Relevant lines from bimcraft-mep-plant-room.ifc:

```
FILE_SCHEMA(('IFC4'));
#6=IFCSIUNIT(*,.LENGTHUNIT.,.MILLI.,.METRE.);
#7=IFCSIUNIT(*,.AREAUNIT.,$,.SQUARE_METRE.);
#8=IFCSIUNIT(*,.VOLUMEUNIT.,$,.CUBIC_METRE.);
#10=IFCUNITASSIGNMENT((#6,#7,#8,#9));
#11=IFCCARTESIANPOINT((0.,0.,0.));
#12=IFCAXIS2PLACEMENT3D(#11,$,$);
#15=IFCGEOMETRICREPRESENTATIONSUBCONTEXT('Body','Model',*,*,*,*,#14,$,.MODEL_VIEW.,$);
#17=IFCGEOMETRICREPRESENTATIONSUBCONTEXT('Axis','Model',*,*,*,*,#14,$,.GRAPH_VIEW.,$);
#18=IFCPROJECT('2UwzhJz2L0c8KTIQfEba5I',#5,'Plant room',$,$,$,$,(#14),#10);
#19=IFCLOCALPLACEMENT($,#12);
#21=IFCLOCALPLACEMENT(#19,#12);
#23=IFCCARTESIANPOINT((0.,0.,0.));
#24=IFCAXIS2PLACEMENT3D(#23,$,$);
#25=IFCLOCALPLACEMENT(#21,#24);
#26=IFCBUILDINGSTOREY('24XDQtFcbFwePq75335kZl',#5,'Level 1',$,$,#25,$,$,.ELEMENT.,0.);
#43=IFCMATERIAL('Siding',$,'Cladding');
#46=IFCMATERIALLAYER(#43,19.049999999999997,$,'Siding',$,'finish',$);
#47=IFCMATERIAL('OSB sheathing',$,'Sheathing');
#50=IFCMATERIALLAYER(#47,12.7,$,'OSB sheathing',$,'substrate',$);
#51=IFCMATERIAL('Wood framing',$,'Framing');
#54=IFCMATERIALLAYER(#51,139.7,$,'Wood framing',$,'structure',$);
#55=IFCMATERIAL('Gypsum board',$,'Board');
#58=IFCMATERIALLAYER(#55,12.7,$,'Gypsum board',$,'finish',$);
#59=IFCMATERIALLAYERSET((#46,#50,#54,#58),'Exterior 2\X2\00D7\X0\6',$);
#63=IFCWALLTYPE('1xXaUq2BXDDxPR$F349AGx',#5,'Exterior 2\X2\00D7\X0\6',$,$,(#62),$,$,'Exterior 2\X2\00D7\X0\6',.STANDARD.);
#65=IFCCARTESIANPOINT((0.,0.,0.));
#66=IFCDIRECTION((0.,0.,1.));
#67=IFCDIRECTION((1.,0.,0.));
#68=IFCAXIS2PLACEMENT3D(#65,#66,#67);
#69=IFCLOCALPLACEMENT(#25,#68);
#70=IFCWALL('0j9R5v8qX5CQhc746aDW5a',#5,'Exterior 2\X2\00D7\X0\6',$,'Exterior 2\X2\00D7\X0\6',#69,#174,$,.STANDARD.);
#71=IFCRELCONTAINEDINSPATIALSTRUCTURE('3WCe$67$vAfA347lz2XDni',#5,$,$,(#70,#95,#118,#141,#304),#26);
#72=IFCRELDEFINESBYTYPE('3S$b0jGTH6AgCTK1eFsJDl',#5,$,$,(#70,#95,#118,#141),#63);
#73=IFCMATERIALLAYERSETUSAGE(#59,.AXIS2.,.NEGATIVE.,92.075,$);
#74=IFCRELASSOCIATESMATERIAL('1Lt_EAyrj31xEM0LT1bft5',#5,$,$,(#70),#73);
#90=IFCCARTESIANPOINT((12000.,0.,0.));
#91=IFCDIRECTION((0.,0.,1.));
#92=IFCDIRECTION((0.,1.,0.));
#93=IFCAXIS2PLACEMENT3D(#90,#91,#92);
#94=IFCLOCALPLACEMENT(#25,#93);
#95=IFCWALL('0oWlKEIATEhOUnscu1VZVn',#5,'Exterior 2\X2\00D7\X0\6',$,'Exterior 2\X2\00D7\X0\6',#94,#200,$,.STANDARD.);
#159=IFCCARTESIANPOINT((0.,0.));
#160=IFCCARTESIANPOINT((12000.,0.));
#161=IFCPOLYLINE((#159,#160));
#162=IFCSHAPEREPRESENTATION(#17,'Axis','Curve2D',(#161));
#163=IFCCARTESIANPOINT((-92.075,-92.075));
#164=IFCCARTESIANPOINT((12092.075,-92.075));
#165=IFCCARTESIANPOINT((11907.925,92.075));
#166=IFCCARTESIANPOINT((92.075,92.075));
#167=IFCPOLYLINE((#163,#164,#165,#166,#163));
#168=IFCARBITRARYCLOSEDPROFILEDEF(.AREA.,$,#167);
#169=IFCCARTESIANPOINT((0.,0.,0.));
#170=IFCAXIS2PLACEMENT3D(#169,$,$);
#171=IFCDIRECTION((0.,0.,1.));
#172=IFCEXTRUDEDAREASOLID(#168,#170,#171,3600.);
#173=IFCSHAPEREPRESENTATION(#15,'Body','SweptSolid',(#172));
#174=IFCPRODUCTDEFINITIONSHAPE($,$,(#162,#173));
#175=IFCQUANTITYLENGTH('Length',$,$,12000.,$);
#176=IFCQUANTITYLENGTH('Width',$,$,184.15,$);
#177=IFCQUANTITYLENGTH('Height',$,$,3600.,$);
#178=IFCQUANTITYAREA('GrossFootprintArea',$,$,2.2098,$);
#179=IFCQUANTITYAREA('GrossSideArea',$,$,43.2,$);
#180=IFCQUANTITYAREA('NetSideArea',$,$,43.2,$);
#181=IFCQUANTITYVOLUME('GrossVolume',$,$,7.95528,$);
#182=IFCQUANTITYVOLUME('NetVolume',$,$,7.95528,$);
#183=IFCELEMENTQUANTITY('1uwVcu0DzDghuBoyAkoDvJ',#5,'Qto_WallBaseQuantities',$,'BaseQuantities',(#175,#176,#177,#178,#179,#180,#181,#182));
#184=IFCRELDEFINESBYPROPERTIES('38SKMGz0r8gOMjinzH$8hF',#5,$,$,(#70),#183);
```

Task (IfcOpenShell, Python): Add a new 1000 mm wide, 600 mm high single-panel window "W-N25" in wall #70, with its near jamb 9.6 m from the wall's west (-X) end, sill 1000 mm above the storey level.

```python
import numpy as np
import ifcopenshell
import ifcopenshell.api.feature
import ifcopenshell.api.geometry
import ifcopenshell.api.pset
import ifcopenshell.api.root
import ifcopenshell.api.spatial
import ifcopenshell.geom
import ifcopenshell.util.element
import ifcopenshell.util.placement
import ifcopenshell.util.representation
import ifcopenshell.util.shape
import ifcopenshell.util.unit

model = ifcopenshell.open("bimcraft-mep-plant-room.ifc")
unit_scale = ifcopenshell.util.unit.calculate_unit_scale(model)
area_scale = ifcopenshell.util.unit.calculate_unit_scale(model, "AREAUNIT")
volume_scale = ifcopenshell.util.unit.calculate_unit_scale(model, "VOLUMEUNIT")
settings = ifcopenshell.geom.settings()


def volume(element):
    """Net volume in cubic metres, openings subtracted."""
    shape = ifcopenshell.geom.create_shape(settings, element)
    return ifcopenshell.util.shape.get_volume(shape.geometry)


wall = model.by_guid("0j9R5v8qX5CQhc746aDW5a")
storey = ifcopenshell.util.element.get_container(wall, ifc_class="IfcBuildingStorey")
context = ifcopenshell.util.representation.get_context(model, "Model", "Body", "MODEL_VIEW")
before = volume(wall)

width, height, from_end, sill = 1, 0.6, 9.6, 1  # metres

# The wall runs along its own X axis, and the end named is its -X end.
wall_shape = ifcopenshell.geom.create_shape(settings, wall)
x, y, z = ifcopenshell.util.shape.get_vertices(wall_shape.geometry).T
start = x.min() + from_end
face, thickness = float(y.min()), float(y.max() - y.min())
wall_matrix = ifcopenshell.util.placement.get_local_placement(wall.ObjectPlacement)
level = ifcopenshell.util.placement.get_local_placement(storey.ObjectPlacement)[2, 3]


def in_wall(x, y):
    """Placement at x, y metres in the wall's axes, at sill height."""
    matrix = wall_matrix.copy()
    matrix[:, 3] = wall_matrix @ np.array([x / unit_scale, y / unit_scale, 0.0, 1.0])
    matrix[2, 3] = level + sill / unit_scale
    return matrix


# Opening: a box that overshoots both wall faces by 50 mm.
opening = ifcopenshell.api.root.create_entity(model, ifc_class="IfcOpeningElement", predefined_type="OPENING")
box = ifcopenshell.api.geometry.add_wall_representation(
    model, context=context, length=width, height=height, thickness=thickness + 0.1
)
ifcopenshell.api.geometry.assign_representation(model, product=opening, representation=box)
ifcopenshell.api.geometry.edit_object_placement(model, product=opening, matrix=in_wall(start, face - 0.05), is_si=False)
ifcopenshell.api.feature.add_feature(model, feature=opening, element=wall)

window = ifcopenshell.api.root.create_entity(model, ifc_class="IfcWindow", name="W-N25", predefined_type="WINDOW")
window.OverallWidth, window.OverallHeight = width / unit_scale, height / unit_scale
window.PartitioningType = "SINGLE_PANEL"
body = ifcopenshell.api.geometry.add_window_representation(
    model,
    context=context,
    overall_width=window.OverallWidth,
    overall_height=window.OverallHeight,
    partition_type="SINGLE_PANEL",
)
ifcopenshell.api.geometry.assign_representation(model, product=window, representation=body)
ifcopenshell.api.spatial.assign_container(model, products=[window], relating_structure=storey)
ifcopenshell.api.feature.add_filling(model, opening=opening, element=window)

# Centre the window in the wall's thickness.
ifcopenshell.api.geometry.edit_object_placement(model, product=window, matrix=in_wall(start, face), is_si=False)
window_shape = ifcopenshell.geom.create_shape(settings, window)
depth = ifcopenshell.util.shape.get_vertices(window_shape.geometry)[:, 1]
offset = face + thickness / 2 - (depth.min() + depth.max()) / 2
ifcopenshell.api.geometry.edit_object_placement(model, product=window, matrix=in_wall(start, offset), is_si=False)

after = volume(wall)

# Update the wall's stored quantities.
qto = model.by_id(ifcopenshell.util.element.get_pset(wall, "Qto_WallBaseQuantities", should_inherit=False)["id"])
ifcopenshell.api.pset.edit_qto(model, qto=qto, properties={
    "NetSideArea": after / thickness / area_scale,
    "NetVolume": after / volume_scale,
})

print(f"wall volume {before:.3f} -> {after:.3f} m3")

model.write("bimcraft-mep-plant-room_v2.ifc")
```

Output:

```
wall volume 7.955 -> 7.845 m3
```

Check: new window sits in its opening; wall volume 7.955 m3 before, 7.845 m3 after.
